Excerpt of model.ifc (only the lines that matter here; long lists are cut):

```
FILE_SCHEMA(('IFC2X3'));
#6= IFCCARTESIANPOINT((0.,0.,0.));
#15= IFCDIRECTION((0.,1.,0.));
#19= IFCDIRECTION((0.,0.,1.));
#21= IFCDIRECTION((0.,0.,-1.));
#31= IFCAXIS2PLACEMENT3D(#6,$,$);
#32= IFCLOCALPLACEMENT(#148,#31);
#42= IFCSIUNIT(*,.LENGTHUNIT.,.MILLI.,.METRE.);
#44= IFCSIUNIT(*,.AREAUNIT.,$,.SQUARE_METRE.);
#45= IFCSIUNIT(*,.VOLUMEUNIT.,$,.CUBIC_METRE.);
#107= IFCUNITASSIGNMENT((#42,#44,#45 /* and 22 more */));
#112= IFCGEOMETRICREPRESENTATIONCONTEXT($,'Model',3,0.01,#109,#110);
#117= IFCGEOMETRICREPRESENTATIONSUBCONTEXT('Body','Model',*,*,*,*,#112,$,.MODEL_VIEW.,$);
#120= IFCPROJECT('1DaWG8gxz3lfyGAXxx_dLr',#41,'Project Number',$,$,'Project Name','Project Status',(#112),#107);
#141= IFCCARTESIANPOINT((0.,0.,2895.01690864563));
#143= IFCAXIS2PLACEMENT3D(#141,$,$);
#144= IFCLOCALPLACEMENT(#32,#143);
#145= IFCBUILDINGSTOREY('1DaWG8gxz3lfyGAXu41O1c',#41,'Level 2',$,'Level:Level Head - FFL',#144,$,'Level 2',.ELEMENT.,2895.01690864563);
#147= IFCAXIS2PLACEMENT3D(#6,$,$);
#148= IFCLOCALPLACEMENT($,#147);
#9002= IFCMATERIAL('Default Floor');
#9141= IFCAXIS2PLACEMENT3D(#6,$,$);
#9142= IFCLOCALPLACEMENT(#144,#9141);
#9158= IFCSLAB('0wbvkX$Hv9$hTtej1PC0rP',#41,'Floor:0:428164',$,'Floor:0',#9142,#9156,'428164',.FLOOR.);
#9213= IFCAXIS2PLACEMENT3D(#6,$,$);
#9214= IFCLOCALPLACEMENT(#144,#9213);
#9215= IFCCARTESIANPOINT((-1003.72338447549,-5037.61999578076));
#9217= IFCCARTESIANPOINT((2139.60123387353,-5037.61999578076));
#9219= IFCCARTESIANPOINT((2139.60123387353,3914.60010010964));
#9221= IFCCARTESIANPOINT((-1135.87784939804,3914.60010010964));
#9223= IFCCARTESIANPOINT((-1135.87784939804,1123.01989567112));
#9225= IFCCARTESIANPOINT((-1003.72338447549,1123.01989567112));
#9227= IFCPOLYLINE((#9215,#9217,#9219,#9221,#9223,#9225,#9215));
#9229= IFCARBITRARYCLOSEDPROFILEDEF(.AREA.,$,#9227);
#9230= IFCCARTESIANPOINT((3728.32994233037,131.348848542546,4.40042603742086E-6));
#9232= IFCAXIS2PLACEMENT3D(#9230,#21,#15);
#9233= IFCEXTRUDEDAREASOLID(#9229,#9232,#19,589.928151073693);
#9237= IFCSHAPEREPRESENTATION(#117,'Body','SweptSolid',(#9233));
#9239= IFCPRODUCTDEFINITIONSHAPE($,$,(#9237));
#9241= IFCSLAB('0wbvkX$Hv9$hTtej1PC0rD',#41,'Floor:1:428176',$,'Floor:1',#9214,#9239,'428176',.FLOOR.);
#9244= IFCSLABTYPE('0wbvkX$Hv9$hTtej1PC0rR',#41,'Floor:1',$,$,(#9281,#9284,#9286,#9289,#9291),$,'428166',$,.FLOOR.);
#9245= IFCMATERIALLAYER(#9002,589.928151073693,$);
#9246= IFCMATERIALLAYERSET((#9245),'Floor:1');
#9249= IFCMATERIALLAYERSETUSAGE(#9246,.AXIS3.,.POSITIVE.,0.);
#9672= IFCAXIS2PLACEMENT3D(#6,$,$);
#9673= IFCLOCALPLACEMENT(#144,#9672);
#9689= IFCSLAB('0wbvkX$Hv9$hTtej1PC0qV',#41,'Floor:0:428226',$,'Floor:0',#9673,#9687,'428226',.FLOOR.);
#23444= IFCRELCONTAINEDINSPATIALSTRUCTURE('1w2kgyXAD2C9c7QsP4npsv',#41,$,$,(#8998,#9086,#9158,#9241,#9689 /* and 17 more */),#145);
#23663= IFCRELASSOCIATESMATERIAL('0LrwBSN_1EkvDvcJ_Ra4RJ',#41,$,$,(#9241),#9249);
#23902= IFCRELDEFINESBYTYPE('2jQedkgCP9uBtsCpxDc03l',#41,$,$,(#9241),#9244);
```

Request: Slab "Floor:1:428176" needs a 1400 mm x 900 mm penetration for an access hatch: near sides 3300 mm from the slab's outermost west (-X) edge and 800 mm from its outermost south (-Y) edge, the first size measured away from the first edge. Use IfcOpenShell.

```python
import numpy as np
import ifcopenshell
import ifcopenshell.api.feature
import ifcopenshell.api.geometry
import ifcopenshell.api.root
import ifcopenshell.geom
import ifcopenshell.util.placement
import ifcopenshell.util.representation
import ifcopenshell.util.shape
import ifcopenshell.util.unit

model = ifcopenshell.open("model.ifc")
unit_scale = ifcopenshell.util.unit.calculate_unit_scale(model)
settings = ifcopenshell.geom.settings()


def volume(element):
    """Net volume in cubic metres, openings subtracted."""
    shape = ifcopenshell.geom.create_shape(settings, element)
    return ifcopenshell.util.shape.get_volume(shape.geometry)


slab = model.by_guid("0wbvkX$Hv9$hTtej1PC0rD")
before = volume(slab)

# Extent in the slab's own axes, in metres. The edges named are its -X and -Y sides.
slab_shape = ifcopenshell.geom.create_shape(settings, slab)
vertices = ifcopenshell.util.shape.get_vertices(slab_shape.geometry)
x_min, y_min, bottom = vertices.min(axis=0)
top = vertices[:, 2].max()

opening = ifcopenshell.api.root.create_entity(model, ifc_class="IfcOpeningElement", name="Access hatch opening")
context = ifcopenshell.util.representation.get_context(model, "Model", "Body", "MODEL_VIEW")
width, depth = 1.4, 0.9
outline = [(0.0, 0.0), (width, 0.0), (width, depth), (0.0, depth), (0.0, 0.0)]
# Overshoot both faces by 50 mm so the cut is clean.
shape = ifcopenshell.api.geometry.add_slab_representation(
    model, context=context, depth=top - bottom + 0.1, polyline=outline
)
ifcopenshell.api.geometry.assign_representation(model, product=opening, representation=shape)

matrix = ifcopenshell.util.placement.get_local_placement(slab.ObjectPlacement)
matrix[:, 3] = matrix @ np.append(np.array([x_min + 3.3, y_min + 0.8, bottom - 0.05]) / unit_scale, 1.0)
ifcopenshell.api.geometry.edit_object_placement(model, product=opening, matrix=matrix, is_si=False)
ifcopenshell.api.feature.add_feature(model, feature=opening, element=slab)

after = volume(slab)

print(f"slab volume {before:.3f} -> {after:.3f} m3")

model.write("model_updated.ifc")
```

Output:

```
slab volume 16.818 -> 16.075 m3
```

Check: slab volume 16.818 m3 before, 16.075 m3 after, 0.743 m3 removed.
